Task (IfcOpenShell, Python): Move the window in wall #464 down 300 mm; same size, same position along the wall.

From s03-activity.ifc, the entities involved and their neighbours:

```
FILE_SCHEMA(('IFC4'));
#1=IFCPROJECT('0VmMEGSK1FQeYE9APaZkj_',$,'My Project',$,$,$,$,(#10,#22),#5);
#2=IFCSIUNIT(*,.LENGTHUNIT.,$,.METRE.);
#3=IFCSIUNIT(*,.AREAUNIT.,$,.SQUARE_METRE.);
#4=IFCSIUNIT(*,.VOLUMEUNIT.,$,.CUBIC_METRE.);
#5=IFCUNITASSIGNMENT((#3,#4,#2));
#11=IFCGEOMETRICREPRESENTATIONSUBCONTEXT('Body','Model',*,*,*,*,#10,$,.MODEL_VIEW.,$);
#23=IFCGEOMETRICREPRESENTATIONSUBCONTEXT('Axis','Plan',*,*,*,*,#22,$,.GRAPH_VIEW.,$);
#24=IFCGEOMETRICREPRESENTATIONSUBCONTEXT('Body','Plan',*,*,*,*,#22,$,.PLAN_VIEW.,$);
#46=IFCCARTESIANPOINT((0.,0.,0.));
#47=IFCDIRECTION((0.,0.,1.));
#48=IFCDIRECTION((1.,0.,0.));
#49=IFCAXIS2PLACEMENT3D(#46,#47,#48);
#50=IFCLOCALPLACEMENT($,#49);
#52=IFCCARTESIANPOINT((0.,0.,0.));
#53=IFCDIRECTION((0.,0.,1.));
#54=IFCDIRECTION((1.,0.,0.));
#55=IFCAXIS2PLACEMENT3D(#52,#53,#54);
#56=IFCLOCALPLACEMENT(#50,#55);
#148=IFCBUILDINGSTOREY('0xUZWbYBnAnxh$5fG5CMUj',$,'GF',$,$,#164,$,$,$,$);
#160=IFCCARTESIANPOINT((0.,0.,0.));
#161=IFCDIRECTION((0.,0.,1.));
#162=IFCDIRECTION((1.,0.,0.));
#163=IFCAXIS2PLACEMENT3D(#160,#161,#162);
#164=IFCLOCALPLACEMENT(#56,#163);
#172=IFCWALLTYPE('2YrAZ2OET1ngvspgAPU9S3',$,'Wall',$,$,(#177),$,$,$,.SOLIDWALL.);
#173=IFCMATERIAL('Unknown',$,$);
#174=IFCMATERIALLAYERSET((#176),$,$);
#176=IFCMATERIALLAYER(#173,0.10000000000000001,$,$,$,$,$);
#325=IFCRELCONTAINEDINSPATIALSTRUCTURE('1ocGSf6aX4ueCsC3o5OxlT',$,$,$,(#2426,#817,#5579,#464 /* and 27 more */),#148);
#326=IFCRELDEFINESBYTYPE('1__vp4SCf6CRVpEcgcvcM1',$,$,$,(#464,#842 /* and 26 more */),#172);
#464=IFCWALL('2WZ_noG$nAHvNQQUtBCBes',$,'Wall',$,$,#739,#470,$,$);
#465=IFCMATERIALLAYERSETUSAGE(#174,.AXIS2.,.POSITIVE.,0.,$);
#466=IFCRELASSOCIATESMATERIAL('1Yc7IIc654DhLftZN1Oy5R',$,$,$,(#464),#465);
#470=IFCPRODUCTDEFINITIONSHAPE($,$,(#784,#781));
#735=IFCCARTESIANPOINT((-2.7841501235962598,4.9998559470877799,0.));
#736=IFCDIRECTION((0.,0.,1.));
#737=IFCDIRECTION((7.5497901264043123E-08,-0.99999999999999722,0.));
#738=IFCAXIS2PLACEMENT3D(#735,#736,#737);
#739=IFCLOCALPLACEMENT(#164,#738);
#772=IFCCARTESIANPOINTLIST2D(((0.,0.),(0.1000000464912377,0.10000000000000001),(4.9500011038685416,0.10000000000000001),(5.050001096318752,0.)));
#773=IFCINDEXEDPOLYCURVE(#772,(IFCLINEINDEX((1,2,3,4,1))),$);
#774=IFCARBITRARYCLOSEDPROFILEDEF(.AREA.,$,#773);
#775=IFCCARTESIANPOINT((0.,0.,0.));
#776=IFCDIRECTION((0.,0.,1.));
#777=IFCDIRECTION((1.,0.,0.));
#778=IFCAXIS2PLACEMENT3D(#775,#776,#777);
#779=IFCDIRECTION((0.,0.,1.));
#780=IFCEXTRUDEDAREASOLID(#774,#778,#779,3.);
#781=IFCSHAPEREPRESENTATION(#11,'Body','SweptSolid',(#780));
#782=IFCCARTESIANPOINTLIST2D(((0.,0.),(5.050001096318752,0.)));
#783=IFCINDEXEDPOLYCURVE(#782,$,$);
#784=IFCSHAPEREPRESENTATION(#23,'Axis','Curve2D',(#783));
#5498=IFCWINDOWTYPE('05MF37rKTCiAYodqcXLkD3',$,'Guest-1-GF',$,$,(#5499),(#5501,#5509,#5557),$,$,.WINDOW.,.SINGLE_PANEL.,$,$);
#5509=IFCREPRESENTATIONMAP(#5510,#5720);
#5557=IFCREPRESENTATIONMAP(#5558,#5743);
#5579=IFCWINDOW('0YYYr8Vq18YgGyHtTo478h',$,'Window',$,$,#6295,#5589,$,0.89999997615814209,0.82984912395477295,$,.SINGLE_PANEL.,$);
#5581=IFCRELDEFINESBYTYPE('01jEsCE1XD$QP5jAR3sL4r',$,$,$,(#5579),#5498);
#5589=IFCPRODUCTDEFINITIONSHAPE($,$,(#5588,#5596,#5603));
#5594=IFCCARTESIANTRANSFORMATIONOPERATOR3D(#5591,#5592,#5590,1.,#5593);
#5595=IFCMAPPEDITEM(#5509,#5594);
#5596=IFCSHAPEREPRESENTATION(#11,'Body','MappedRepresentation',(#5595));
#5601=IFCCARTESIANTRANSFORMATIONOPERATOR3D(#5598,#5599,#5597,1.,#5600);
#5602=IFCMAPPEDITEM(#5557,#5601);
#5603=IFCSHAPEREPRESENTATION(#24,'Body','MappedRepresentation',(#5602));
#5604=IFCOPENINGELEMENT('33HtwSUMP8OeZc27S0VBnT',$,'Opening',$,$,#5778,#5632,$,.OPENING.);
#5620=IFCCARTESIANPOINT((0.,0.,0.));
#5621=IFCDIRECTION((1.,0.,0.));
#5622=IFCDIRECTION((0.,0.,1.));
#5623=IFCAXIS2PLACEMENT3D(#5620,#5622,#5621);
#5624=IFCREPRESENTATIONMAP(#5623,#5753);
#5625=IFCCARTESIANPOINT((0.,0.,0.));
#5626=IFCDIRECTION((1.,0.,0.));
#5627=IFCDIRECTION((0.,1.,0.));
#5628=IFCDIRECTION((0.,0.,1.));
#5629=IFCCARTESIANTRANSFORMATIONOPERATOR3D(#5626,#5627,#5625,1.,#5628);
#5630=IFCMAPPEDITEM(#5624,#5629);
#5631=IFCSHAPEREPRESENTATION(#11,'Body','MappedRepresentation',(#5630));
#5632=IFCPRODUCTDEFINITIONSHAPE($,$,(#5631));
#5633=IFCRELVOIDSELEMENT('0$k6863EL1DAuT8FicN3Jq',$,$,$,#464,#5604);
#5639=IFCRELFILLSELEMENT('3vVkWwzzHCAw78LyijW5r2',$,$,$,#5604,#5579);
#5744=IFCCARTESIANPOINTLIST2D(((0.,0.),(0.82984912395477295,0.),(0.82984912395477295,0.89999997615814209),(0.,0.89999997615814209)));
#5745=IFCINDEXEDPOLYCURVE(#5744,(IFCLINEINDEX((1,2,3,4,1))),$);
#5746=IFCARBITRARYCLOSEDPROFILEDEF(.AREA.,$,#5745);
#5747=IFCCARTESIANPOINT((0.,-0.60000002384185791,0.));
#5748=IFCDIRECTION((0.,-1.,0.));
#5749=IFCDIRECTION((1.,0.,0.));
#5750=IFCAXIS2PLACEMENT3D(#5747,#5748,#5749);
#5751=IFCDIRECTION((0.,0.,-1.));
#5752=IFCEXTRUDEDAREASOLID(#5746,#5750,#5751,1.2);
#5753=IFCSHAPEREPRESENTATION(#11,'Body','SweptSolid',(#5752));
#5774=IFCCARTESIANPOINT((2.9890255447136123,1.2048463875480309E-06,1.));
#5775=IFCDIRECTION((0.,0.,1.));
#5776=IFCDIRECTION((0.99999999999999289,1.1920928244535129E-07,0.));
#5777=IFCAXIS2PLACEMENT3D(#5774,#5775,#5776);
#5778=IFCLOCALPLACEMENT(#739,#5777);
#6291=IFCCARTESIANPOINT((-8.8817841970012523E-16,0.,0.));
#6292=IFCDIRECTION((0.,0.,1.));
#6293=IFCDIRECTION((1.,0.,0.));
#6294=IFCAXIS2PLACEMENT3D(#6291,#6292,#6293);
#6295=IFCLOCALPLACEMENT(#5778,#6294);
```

```python
import numpy as np
import ifcopenshell
import ifcopenshell.api.geometry
import ifcopenshell.util.placement
import ifcopenshell.util.unit

model = ifcopenshell.open("s03-activity.ifc")
unit_scale = ifcopenshell.util.unit.calculate_unit_scale(model)

window = model.by_guid("0YYYr8Vq18YgGyHtTo478h")
opening = window.FillsVoids[0].RelatingOpeningElement
dz = -0.3

shift = np.array([0.0, 0.0, dz])
# The window is placed relative to its opening, so it follows when the opening moves.
matrix = ifcopenshell.util.placement.get_local_placement(opening.ObjectPlacement)
matrix[:3, 3] += shift
ifcopenshell.api.geometry.edit_object_placement(
    model, product=opening, matrix=matrix, is_si=False, should_transform_children=True
)

print(f"moved by {dz * unit_scale:+.3f} m")

model.write("s03-activity_edited.ifc")
```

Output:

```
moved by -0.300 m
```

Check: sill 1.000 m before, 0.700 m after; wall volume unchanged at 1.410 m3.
